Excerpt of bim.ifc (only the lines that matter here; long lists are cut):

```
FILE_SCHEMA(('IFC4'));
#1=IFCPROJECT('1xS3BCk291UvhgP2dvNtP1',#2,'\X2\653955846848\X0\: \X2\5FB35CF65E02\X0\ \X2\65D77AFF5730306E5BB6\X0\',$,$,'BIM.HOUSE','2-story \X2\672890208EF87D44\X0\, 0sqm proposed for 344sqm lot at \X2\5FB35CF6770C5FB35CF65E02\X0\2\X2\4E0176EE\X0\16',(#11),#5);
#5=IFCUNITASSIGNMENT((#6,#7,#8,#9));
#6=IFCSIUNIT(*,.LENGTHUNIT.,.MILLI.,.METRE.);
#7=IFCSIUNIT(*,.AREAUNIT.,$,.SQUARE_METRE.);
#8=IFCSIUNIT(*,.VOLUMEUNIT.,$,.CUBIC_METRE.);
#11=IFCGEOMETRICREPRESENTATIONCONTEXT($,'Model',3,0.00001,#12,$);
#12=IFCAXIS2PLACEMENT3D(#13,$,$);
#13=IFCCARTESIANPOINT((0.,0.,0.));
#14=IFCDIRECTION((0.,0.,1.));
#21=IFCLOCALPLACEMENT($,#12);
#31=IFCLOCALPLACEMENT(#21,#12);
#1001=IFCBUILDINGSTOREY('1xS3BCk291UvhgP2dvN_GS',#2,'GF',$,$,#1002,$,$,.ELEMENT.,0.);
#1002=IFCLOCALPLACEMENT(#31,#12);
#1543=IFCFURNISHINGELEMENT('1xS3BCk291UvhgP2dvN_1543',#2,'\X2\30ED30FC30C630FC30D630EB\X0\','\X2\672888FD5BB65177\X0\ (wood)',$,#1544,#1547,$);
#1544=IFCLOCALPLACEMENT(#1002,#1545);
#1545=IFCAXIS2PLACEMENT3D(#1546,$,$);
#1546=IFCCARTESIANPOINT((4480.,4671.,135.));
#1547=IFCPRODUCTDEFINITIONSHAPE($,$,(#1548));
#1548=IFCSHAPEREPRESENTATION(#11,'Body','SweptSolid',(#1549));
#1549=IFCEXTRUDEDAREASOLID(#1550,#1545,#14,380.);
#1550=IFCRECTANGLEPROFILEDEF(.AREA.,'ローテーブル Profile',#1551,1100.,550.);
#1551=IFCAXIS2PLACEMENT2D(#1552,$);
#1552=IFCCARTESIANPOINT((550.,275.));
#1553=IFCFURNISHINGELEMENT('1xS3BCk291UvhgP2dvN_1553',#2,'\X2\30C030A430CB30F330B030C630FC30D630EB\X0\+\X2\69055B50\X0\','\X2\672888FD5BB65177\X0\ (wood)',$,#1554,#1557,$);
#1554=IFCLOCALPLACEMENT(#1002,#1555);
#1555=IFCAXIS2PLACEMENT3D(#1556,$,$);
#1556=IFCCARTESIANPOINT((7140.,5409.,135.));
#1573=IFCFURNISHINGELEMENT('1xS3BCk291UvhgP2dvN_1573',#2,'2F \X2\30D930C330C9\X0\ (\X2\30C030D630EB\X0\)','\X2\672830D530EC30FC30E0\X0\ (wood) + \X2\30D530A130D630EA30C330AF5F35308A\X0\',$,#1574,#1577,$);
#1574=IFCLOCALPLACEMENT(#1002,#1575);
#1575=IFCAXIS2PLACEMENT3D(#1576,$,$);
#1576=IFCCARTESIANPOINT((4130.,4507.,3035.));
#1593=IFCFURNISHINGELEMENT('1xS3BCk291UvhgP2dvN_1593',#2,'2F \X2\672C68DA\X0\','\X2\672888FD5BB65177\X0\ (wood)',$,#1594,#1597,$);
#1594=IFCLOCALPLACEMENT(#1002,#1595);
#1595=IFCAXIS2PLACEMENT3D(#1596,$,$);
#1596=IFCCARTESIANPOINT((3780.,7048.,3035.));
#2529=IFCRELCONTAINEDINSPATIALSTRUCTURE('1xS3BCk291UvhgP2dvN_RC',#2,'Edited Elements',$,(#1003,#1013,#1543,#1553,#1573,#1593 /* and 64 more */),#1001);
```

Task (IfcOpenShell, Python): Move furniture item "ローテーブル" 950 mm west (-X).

```python
import ifcopenshell
import ifcopenshell.api.geometry
import ifcopenshell.util.placement
import ifcopenshell.util.unit

model = ifcopenshell.open("bim.ifc")
unit_scale = ifcopenshell.util.unit.calculate_unit_scale(model)

item = model.by_guid("1xS3BCk291UvhgP2dvN_1543")
matrix = ifcopenshell.util.placement.get_local_placement(item.ObjectPlacement)
matrix[0, 3] -= 0.95 / unit_scale
ifcopenshell.api.geometry.edit_object_placement(model, product=item, matrix=matrix, is_si=False)

print(ifcopenshell.util.placement.get_local_placement(item.ObjectPlacement).round(3) + 0.0)

model.write("bim_rev.ifc")
```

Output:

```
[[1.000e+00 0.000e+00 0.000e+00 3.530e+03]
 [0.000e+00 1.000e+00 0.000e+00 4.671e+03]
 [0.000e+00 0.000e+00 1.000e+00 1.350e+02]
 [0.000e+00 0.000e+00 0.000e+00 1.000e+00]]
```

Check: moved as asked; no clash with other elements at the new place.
